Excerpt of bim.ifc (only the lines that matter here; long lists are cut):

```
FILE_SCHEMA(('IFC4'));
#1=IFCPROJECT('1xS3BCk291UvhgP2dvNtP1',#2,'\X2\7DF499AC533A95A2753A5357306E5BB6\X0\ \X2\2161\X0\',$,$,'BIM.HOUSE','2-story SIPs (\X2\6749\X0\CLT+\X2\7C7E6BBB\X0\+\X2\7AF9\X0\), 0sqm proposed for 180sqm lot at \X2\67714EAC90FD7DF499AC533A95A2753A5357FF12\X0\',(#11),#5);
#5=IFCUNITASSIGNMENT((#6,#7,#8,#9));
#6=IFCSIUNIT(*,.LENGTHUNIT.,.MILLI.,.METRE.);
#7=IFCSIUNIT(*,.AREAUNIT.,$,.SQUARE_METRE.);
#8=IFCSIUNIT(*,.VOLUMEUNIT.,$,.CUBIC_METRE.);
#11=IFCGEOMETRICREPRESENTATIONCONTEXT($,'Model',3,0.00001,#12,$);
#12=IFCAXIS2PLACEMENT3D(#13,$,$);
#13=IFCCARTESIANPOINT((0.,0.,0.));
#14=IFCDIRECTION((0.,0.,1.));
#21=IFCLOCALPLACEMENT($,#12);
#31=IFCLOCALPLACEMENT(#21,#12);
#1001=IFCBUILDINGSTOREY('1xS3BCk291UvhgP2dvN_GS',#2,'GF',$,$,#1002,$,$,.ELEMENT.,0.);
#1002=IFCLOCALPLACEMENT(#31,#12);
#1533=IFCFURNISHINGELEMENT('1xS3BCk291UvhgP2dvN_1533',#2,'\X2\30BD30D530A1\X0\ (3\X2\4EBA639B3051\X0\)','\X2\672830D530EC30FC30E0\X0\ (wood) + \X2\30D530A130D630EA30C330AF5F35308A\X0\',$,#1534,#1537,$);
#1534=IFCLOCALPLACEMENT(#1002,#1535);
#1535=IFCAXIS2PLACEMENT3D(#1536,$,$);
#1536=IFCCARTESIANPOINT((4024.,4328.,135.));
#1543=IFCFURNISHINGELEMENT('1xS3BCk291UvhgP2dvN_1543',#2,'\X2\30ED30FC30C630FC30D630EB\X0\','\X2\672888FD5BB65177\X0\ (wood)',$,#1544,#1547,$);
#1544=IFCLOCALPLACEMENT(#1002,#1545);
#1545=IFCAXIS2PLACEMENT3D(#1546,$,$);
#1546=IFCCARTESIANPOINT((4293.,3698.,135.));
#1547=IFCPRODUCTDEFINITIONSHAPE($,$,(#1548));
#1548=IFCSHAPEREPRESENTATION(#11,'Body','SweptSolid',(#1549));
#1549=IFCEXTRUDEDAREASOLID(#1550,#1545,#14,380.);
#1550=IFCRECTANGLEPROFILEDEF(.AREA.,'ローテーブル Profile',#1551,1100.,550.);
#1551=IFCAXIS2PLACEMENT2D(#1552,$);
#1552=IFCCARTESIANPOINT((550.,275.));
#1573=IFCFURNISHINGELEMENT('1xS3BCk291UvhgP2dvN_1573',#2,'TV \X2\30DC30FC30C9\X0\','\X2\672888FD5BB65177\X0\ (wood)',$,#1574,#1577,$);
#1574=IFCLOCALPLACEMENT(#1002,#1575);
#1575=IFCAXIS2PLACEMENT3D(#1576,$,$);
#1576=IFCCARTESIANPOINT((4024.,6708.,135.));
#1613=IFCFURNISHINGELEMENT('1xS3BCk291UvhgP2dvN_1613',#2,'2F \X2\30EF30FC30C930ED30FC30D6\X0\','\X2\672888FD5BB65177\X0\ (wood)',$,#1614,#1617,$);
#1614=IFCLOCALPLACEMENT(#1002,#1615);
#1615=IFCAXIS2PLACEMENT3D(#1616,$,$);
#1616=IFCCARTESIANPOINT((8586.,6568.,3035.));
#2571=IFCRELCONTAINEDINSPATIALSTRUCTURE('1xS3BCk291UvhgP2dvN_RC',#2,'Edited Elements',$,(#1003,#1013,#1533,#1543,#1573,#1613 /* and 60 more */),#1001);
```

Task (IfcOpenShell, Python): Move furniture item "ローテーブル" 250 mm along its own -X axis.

```python
import ifcopenshell
import ifcopenshell.api.geometry
import ifcopenshell.util.placement
import ifcopenshell.util.unit

model = ifcopenshell.open("bim.ifc")
unit_scale = ifcopenshell.util.unit.calculate_unit_scale(model)

item = model.by_guid("1xS3BCk291UvhgP2dvN_1543")
matrix = ifcopenshell.util.placement.get_local_placement(item.ObjectPlacement)
matrix[:3, 3] -= matrix[:3, 0] * 0.25 / unit_scale
ifcopenshell.api.geometry.edit_object_placement(model, product=item, matrix=matrix, is_si=False)

print(ifcopenshell.util.placement.get_local_placement(item.ObjectPlacement).round(3) + 0.0)

model.write("bim_v2.ifc")
```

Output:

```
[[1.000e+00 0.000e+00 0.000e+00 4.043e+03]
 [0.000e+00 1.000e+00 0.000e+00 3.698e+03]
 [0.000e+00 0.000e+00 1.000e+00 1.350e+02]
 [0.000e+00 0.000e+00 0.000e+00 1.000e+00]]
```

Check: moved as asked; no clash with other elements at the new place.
